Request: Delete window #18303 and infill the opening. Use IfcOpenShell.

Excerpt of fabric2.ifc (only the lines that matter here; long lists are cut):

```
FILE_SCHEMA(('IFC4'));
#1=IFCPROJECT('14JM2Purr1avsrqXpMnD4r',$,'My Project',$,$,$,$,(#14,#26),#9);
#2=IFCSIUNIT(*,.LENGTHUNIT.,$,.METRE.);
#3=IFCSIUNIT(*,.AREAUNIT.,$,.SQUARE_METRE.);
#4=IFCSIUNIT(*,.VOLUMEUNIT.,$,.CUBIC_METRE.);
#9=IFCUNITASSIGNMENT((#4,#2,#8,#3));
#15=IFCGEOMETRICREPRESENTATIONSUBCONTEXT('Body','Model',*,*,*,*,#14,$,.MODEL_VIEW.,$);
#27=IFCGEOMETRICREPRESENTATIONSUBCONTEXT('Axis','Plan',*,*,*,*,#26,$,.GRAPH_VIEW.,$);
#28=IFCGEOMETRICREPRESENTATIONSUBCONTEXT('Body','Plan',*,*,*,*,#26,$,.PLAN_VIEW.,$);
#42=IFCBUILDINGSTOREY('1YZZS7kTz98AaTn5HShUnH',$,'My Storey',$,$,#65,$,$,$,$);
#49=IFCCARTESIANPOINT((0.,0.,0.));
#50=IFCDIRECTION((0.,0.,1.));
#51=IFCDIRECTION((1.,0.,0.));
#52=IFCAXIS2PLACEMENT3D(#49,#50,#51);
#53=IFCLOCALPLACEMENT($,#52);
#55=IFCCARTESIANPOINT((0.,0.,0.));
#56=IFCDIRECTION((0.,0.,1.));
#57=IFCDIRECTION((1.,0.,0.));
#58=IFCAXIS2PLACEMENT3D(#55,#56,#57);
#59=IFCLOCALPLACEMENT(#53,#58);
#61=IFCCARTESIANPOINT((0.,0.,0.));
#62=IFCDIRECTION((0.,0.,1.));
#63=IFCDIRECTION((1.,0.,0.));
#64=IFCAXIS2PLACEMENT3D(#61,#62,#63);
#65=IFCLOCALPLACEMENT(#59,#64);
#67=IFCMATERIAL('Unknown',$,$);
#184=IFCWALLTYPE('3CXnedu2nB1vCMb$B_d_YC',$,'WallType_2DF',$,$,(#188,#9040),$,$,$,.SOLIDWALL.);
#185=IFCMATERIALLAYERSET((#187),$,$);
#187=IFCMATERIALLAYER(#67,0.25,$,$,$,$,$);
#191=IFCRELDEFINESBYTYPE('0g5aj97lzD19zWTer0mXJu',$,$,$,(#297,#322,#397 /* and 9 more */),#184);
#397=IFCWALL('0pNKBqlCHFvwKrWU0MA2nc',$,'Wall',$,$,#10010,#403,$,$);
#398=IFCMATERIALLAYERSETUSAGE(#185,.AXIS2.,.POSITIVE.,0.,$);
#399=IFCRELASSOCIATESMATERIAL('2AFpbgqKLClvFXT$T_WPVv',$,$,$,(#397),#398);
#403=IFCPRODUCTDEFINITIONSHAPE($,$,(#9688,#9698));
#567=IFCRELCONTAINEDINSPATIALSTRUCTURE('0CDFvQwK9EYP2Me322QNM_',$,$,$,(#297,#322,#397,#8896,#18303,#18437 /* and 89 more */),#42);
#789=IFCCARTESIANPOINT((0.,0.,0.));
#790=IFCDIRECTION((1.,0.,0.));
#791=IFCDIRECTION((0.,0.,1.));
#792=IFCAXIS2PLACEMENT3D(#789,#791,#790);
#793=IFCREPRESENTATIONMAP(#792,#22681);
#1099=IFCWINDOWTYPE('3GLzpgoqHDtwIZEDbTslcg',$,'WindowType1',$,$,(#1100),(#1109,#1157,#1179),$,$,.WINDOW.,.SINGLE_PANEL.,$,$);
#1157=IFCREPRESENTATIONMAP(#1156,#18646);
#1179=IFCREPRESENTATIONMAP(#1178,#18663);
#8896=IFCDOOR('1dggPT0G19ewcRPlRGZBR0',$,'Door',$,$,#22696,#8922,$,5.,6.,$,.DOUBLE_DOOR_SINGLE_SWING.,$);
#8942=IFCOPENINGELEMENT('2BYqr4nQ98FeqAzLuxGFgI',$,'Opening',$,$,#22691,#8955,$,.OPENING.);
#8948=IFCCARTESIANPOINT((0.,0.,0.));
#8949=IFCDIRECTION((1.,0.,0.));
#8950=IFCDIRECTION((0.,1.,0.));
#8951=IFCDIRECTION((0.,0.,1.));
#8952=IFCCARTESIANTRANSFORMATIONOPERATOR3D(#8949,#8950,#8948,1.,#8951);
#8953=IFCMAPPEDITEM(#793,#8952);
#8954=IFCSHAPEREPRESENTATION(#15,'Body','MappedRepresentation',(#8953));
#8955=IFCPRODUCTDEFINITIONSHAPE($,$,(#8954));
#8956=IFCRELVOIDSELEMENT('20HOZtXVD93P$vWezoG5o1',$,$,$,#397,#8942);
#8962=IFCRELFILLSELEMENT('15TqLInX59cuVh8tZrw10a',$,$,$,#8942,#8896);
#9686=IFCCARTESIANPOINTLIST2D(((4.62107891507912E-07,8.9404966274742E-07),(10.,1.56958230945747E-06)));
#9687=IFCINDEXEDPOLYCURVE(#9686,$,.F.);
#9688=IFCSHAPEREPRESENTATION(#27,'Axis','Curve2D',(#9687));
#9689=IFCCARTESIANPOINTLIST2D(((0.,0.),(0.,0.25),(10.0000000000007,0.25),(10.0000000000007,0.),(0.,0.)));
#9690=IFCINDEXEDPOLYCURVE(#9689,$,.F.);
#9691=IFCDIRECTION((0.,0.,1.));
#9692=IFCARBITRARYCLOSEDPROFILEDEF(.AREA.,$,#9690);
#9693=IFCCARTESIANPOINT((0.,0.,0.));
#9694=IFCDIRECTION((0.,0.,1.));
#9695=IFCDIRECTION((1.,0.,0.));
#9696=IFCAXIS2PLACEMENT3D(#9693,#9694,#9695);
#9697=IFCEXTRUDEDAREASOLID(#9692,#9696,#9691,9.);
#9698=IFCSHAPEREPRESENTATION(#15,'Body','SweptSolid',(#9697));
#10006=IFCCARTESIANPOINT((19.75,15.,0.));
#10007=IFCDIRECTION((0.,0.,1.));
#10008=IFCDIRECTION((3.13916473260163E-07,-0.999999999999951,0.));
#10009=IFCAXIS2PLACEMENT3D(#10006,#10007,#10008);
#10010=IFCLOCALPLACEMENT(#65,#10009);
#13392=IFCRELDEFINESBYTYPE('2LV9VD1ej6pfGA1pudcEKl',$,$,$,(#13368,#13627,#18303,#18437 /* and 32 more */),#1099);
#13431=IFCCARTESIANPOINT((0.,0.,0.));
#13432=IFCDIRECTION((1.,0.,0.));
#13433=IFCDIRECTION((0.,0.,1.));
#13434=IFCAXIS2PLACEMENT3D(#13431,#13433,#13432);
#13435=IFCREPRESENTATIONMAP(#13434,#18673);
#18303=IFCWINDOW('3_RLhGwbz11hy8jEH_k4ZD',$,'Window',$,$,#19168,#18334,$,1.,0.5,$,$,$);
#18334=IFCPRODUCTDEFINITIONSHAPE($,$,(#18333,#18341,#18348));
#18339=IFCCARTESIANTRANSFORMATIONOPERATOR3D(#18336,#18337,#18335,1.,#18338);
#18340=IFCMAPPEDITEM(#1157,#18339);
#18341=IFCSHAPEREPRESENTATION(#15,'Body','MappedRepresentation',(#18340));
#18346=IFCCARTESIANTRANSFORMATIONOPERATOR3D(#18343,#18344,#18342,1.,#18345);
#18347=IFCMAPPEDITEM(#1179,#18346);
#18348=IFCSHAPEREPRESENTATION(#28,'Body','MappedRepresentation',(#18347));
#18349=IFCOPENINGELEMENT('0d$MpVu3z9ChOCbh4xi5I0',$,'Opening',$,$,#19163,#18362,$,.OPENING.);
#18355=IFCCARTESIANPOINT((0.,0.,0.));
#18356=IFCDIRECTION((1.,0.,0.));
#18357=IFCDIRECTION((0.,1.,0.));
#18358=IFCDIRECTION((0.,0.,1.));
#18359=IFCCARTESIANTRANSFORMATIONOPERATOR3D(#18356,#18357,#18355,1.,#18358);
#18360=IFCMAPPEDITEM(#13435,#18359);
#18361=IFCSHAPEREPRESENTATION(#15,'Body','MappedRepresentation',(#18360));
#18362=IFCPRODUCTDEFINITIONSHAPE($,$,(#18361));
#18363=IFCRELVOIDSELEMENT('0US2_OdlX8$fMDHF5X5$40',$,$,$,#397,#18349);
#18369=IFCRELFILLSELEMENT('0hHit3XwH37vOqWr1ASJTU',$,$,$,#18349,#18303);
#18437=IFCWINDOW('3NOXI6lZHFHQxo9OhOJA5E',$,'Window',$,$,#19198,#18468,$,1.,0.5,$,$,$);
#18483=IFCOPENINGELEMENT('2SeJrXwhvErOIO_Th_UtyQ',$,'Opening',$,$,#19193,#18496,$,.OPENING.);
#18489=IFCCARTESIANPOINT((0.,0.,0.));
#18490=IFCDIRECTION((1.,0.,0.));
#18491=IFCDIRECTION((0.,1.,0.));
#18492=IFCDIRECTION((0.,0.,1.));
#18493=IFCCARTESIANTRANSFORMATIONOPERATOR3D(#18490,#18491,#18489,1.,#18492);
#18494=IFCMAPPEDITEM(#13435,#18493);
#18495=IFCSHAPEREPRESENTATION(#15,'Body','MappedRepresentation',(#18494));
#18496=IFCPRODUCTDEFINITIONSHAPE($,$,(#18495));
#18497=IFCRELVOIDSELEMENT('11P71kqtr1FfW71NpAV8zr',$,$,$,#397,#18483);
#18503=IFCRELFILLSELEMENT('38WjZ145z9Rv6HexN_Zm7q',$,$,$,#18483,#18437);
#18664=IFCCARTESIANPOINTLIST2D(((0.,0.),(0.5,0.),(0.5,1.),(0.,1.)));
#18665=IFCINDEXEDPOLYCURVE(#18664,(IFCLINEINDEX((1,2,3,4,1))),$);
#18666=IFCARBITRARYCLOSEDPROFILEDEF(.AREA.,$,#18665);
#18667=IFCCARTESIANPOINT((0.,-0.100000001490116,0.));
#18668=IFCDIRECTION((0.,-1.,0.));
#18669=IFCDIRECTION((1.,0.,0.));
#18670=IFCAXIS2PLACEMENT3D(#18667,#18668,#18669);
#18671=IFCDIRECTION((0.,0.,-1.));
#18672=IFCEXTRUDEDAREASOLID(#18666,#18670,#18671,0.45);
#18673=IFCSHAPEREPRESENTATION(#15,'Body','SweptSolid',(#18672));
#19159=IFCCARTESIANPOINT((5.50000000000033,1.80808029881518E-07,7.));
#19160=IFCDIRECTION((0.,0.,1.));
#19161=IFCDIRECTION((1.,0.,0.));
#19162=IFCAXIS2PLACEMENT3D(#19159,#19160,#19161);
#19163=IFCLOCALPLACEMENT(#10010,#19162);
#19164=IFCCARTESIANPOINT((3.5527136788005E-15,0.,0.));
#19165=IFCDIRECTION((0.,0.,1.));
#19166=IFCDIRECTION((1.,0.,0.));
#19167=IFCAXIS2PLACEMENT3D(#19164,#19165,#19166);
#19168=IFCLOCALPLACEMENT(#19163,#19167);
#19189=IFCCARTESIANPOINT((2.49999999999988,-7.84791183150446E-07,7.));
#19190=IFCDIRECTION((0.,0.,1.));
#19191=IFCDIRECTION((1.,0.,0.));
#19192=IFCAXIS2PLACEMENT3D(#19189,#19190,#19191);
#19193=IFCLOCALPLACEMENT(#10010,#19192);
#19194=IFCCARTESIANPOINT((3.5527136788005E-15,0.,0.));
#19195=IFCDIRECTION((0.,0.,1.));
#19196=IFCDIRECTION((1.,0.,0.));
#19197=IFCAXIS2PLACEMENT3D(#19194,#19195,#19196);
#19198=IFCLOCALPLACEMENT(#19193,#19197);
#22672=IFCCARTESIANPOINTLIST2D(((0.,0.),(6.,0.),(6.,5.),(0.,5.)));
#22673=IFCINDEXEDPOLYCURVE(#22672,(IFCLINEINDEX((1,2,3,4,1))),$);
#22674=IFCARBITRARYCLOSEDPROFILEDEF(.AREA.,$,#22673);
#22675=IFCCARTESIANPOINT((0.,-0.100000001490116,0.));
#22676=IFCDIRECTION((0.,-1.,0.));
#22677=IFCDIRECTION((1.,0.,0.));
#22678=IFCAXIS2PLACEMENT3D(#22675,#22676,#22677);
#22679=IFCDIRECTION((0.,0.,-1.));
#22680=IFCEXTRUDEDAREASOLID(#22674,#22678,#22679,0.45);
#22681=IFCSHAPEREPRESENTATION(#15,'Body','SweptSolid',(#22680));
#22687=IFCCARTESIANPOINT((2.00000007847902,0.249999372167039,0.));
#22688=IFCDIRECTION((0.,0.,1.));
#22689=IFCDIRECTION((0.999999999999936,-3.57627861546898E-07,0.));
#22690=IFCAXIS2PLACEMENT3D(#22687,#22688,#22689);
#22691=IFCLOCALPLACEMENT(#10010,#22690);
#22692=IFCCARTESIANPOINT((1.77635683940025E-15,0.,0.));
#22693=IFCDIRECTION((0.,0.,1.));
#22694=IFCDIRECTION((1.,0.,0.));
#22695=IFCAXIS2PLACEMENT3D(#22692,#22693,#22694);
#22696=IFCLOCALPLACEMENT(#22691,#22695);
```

```python
import ifcopenshell
import ifcopenshell.api.feature
import ifcopenshell.api.root
import ifcopenshell.geom
import ifcopenshell.util.shape

model = ifcopenshell.open("fabric2.ifc")
settings = ifcopenshell.geom.settings()


def volume(element):
    """Net volume in cubic metres, openings subtracted."""
    shape = ifcopenshell.geom.create_shape(settings, element)
    return ifcopenshell.util.shape.get_volume(shape.geometry)


window = model.by_guid("3_RLhGwbz11hy8jEH_k4ZD")
opening = window.FillsVoids[0].RelatingOpeningElement
wall = opening.VoidsElements[0].RelatingBuildingElement
before = volume(wall)

ifcopenshell.api.root.remove_product(model, product=window)
ifcopenshell.api.feature.remove_feature(model, feature=opening)

after = volume(wall)

print(f"wall volume {before:.3f} -> {after:.3f} m3")

model.write("fabric2_rev.ifc")
```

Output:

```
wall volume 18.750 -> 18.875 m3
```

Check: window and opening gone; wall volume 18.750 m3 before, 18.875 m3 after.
